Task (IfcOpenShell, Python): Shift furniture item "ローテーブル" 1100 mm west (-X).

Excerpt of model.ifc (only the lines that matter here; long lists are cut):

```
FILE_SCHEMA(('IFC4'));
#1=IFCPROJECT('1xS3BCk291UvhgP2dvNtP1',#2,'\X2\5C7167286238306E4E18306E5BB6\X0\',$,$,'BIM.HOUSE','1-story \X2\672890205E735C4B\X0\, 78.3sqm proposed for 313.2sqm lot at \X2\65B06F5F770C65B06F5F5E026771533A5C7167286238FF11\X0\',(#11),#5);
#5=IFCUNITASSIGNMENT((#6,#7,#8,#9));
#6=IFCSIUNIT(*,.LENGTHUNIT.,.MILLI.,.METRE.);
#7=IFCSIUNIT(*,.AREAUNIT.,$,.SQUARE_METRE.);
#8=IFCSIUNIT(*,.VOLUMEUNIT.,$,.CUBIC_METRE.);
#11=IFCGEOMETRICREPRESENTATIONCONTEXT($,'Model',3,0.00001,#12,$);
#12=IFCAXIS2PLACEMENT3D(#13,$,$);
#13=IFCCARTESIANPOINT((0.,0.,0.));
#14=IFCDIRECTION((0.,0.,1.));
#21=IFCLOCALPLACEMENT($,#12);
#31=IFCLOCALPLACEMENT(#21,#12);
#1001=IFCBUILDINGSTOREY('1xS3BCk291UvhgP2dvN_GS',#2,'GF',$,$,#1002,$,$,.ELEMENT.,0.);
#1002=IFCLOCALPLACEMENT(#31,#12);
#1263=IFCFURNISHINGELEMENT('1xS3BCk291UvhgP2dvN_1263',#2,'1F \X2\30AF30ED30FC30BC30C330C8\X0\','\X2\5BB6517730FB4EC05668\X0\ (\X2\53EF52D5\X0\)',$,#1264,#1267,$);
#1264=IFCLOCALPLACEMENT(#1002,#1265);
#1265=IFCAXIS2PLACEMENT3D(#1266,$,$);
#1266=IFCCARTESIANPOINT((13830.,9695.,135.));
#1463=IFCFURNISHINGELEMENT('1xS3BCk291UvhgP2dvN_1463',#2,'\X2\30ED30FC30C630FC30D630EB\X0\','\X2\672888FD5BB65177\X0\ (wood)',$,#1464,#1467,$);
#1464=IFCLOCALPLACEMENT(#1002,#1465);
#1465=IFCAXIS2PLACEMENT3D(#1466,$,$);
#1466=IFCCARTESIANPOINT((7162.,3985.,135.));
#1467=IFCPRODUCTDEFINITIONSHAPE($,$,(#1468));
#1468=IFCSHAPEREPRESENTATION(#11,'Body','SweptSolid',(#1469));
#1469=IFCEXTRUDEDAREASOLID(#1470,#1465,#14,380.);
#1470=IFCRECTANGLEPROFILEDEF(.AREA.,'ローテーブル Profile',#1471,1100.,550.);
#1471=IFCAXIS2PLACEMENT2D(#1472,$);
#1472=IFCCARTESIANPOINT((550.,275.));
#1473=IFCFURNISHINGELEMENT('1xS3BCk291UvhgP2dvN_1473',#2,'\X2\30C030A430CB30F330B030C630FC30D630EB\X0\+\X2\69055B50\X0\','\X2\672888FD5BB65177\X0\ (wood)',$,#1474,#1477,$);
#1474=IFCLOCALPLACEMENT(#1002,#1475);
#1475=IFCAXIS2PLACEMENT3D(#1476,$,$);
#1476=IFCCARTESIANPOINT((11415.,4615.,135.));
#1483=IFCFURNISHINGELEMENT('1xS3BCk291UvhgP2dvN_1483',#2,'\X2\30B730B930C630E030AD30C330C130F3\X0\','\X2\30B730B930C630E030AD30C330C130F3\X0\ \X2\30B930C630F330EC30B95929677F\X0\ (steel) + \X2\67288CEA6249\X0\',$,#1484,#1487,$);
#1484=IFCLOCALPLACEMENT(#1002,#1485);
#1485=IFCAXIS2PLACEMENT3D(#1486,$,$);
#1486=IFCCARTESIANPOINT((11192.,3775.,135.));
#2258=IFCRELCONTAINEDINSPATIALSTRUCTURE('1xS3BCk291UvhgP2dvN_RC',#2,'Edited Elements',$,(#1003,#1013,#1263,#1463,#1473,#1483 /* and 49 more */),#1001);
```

```python
import ifcopenshell
import ifcopenshell.api.geometry
import ifcopenshell.util.placement
import ifcopenshell.util.unit

model = ifcopenshell.open("model.ifc")
unit_scale = ifcopenshell.util.unit.calculate_unit_scale(model)

item = model.by_guid("1xS3BCk291UvhgP2dvN_1463")
matrix = ifcopenshell.util.placement.get_local_placement(item.ObjectPlacement)
matrix[0, 3] -= 1.1 / unit_scale
ifcopenshell.api.geometry.edit_object_placement(model, product=item, matrix=matrix, is_si=False)

print(ifcopenshell.util.placement.get_local_placement(item.ObjectPlacement).round(3) + 0.0)

model.write("model_updated.ifc")
```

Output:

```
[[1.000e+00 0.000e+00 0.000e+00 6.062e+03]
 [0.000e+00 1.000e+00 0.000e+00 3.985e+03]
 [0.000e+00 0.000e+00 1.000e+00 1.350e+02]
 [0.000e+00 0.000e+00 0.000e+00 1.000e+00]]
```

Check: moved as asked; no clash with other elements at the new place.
